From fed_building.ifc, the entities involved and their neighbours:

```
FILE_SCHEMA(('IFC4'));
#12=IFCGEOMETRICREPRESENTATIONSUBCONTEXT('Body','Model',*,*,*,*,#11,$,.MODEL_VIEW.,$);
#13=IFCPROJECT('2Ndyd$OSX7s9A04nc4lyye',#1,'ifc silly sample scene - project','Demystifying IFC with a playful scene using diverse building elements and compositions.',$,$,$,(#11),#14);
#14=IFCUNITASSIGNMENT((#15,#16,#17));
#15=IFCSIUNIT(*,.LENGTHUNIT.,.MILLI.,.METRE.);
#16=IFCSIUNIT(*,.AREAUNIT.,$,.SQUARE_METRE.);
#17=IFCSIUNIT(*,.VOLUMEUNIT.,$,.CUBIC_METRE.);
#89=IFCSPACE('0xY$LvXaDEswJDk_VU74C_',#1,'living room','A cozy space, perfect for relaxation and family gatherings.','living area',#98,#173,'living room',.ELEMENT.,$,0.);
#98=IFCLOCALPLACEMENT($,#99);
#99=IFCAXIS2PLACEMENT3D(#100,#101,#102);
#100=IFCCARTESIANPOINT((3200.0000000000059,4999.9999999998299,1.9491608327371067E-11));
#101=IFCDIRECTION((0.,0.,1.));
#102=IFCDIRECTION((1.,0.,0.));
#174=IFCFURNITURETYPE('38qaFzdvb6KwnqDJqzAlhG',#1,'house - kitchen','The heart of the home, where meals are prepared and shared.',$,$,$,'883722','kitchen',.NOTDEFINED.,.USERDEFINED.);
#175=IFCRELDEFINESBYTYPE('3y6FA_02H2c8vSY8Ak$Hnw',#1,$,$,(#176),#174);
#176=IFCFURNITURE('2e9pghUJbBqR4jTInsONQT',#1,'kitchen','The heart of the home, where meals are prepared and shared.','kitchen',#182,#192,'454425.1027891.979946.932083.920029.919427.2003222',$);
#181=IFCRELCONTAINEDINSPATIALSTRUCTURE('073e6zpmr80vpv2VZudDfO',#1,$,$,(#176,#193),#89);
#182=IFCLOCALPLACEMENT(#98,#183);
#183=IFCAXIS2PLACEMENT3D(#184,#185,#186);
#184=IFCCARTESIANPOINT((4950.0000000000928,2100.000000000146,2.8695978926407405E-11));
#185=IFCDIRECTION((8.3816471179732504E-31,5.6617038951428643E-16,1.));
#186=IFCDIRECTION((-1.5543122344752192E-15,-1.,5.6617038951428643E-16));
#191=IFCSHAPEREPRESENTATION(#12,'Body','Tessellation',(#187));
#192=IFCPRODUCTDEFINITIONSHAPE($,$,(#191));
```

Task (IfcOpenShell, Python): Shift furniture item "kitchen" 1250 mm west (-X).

```python
import ifcopenshell
import ifcopenshell.api.geometry
import ifcopenshell.util.placement

model = ifcopenshell.open("fed_building.ifc")

item = model.by_guid("2e9pghUJbBqR4jTInsONQT")
matrix = ifcopenshell.util.placement.get_local_placement(item.ObjectPlacement)
matrix[0, 3] -= 1250.0
ifcopenshell.api.geometry.edit_object_placement(model, product=item, matrix=matrix, is_si=False)

print(ifcopenshell.util.placement.get_local_placement(item.ObjectPlacement).round(3) + 0.0)

model.write("fed_building_edited.ifc")
```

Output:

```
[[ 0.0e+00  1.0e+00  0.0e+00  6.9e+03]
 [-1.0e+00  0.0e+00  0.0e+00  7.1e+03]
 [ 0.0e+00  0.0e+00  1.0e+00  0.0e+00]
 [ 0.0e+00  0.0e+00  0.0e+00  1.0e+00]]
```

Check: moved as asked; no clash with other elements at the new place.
